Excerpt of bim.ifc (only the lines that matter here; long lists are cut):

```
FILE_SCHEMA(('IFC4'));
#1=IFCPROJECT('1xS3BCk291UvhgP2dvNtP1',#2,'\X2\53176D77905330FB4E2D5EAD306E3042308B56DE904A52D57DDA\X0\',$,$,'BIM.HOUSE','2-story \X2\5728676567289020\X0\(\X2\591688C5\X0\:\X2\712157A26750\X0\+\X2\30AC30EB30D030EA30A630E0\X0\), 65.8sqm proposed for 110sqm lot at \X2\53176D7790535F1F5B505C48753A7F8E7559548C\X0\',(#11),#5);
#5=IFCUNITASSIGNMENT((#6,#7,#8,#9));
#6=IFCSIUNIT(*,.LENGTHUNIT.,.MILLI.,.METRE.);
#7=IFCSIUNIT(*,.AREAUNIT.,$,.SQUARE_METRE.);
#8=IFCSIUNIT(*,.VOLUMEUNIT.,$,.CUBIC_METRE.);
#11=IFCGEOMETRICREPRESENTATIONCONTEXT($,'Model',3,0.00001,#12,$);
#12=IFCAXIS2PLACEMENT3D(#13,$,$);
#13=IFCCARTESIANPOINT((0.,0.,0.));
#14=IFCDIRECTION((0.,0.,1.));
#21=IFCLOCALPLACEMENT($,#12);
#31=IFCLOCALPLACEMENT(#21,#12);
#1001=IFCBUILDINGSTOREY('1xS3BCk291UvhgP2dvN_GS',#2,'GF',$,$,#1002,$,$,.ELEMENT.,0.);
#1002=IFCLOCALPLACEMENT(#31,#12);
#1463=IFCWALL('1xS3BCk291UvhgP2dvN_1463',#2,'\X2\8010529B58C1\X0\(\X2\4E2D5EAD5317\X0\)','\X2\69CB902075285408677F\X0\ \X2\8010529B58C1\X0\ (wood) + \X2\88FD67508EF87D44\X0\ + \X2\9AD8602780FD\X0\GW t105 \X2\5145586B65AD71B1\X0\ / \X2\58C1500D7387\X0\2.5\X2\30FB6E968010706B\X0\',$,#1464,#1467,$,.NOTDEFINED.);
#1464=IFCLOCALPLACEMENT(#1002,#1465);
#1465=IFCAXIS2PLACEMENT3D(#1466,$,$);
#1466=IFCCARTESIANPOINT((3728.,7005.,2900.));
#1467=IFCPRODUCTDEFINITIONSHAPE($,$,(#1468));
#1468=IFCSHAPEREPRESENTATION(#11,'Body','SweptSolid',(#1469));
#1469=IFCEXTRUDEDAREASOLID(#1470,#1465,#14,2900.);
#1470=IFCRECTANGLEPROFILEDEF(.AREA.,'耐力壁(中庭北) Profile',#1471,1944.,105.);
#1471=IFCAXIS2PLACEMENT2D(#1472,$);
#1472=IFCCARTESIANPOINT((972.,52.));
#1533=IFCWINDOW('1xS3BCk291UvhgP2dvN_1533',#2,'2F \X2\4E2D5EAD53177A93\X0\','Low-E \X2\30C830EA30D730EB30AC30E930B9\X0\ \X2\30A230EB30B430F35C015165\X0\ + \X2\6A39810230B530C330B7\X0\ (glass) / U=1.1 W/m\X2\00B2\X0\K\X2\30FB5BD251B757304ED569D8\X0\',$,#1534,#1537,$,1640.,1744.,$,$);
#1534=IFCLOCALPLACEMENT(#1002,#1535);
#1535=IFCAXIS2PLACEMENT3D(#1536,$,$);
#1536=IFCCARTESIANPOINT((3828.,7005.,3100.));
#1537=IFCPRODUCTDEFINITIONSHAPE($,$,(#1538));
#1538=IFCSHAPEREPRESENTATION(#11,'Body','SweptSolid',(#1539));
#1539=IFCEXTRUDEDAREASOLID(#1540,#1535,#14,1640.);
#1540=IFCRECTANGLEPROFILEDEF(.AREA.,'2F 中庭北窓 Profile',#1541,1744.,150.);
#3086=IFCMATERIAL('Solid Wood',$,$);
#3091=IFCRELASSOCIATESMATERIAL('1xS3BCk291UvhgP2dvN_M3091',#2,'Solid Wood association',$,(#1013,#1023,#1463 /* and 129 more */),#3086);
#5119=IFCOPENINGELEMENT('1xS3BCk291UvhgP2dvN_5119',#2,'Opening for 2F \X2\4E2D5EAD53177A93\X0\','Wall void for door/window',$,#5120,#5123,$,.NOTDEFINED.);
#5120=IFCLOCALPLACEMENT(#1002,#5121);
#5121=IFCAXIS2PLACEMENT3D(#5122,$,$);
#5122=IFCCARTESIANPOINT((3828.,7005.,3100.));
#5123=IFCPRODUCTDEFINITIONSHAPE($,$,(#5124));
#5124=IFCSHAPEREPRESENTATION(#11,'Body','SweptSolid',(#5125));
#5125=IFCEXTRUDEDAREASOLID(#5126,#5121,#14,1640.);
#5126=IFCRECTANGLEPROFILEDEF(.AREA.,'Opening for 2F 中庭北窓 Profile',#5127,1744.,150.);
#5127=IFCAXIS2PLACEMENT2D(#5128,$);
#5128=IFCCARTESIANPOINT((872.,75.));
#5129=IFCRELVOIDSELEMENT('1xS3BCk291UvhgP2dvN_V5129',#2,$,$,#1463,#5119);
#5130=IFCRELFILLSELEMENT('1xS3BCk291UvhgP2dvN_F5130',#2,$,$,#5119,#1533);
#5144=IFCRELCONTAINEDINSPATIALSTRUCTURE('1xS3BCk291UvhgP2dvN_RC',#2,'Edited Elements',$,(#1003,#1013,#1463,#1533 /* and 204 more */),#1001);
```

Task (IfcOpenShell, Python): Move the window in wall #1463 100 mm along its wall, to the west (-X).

```python
import ifcopenshell
import ifcopenshell.api.geometry
import ifcopenshell.util.placement
import ifcopenshell.util.unit

model = ifcopenshell.open("bim.ifc")
unit_scale = ifcopenshell.util.unit.calculate_unit_scale(model)

window = model.by_guid("1xS3BCk291UvhgP2dvN_1533")
opening = window.FillsVoids[0].RelatingOpeningElement
wall = opening.VoidsElements[0].RelatingBuildingElement

wall_matrix = ifcopenshell.util.placement.get_local_placement(wall.ObjectPlacement)
shift = wall_matrix[:3, 0] * -0.1 / unit_scale
before = ifcopenshell.util.placement.get_local_placement(window.ObjectPlacement)[:3, 3].copy()

# The window is not placed relative to its opening, so move both.
for product in (opening, window):
    matrix = ifcopenshell.util.placement.get_local_placement(product.ObjectPlacement)
    matrix[:3, 3] += shift
    ifcopenshell.api.geometry.edit_object_placement(model, product=product, matrix=matrix, is_si=False)

after = ifcopenshell.util.placement.get_local_placement(window.ObjectPlacement)[:3, 3]
print("window moved by", (after - before).round(3) + 0.0)

model.write("bim_rev.ifc")
```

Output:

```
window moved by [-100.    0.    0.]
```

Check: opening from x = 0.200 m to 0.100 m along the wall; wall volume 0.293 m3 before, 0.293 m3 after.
